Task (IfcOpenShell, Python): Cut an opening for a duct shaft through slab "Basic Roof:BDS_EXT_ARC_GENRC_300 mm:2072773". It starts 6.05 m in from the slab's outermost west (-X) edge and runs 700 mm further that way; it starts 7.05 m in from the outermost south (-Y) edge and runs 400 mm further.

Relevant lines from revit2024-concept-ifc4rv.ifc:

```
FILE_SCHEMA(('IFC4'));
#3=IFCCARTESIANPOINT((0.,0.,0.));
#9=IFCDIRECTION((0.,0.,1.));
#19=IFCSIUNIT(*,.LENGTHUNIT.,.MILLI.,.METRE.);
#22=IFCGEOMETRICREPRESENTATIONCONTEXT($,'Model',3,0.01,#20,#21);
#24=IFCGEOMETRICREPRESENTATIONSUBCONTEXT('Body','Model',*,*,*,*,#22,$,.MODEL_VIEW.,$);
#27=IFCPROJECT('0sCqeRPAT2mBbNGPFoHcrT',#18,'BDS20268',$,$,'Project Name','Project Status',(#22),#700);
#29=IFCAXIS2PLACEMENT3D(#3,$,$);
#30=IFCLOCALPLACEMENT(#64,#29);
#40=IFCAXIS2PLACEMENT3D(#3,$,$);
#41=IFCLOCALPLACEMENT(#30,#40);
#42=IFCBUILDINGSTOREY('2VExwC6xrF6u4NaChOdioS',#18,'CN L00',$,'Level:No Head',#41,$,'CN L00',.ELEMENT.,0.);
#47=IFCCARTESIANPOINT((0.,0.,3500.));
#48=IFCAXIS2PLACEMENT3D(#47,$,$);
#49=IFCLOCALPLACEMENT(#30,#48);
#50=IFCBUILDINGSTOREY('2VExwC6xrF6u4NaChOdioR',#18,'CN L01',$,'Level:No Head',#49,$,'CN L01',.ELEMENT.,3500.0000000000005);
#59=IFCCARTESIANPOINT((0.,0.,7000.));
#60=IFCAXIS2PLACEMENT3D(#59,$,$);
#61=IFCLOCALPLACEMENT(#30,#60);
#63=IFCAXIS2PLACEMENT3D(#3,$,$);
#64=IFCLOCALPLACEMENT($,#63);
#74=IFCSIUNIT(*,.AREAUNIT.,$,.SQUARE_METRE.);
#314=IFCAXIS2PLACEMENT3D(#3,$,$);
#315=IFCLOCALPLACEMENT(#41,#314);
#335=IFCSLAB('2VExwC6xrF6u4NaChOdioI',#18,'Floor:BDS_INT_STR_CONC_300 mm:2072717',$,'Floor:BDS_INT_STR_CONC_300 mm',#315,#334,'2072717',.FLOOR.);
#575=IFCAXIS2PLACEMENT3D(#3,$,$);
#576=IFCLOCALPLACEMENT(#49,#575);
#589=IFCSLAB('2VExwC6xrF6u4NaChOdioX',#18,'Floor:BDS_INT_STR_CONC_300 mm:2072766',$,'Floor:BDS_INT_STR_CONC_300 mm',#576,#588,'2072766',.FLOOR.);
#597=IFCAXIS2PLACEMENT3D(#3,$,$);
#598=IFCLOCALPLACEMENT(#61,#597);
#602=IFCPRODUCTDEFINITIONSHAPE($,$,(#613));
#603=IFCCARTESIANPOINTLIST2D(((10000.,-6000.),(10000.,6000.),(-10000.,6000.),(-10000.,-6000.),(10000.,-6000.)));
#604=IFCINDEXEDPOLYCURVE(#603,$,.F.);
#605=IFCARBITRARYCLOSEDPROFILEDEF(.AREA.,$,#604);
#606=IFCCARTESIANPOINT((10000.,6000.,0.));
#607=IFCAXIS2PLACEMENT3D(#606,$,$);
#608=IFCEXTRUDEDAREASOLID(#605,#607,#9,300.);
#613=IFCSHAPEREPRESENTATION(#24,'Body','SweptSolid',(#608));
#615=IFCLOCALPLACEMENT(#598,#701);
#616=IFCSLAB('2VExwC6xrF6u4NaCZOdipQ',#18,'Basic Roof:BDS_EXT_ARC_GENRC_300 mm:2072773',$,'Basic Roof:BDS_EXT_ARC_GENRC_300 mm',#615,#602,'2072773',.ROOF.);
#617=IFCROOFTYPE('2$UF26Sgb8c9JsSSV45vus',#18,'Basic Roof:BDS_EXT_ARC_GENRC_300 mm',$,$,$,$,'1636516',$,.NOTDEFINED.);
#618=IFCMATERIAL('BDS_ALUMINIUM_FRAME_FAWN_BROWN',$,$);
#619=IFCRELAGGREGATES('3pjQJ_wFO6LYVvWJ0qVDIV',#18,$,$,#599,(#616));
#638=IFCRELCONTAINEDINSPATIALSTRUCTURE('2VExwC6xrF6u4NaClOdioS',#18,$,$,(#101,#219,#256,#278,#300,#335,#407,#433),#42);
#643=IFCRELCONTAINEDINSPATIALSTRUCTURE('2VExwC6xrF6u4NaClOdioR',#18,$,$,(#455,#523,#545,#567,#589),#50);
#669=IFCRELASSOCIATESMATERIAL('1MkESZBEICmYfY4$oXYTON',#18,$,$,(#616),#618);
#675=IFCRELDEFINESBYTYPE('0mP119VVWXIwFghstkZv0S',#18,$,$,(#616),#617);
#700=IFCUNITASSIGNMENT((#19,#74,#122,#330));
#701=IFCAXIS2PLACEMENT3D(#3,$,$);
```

```python
import numpy as np
import ifcopenshell
import ifcopenshell.api.feature
import ifcopenshell.api.geometry
import ifcopenshell.api.root
import ifcopenshell.geom
import ifcopenshell.util.placement
import ifcopenshell.util.representation
import ifcopenshell.util.shape
import ifcopenshell.util.unit

model = ifcopenshell.open("revit2024-concept-ifc4rv.ifc")
unit_scale = ifcopenshell.util.unit.calculate_unit_scale(model)
settings = ifcopenshell.geom.settings()


def volume(element):
    """Net volume in cubic metres, openings subtracted."""
    shape = ifcopenshell.geom.create_shape(settings, element)
    return ifcopenshell.util.shape.get_volume(shape.geometry)


slab = model.by_guid("2VExwC6xrF6u4NaCZOdipQ")
before = volume(slab)

# Extent in the slab's own axes, in metres. The edges named are its -X and -Y sides.
slab_shape = ifcopenshell.geom.create_shape(settings, slab)
vertices = ifcopenshell.util.shape.get_vertices(slab_shape.geometry)
x_min, y_min, bottom = vertices.min(axis=0)
top = vertices[:, 2].max()

opening = ifcopenshell.api.root.create_entity(model, ifc_class="IfcOpeningElement", name="Duct shaft opening", predefined_type="OPENING")
context = ifcopenshell.util.representation.get_context(model, "Model", "Body", "MODEL_VIEW")
width, depth = 0.7, 0.4
outline = [(0.0, 0.0), (width, 0.0), (width, depth), (0.0, depth), (0.0, 0.0)]
# Overshoot both faces by 50 mm so the cut is clean.
shape = ifcopenshell.api.geometry.add_slab_representation(
    model, context=context, depth=top - bottom + 0.1, polyline=outline
)
ifcopenshell.api.geometry.assign_representation(model, product=opening, representation=shape)

matrix = ifcopenshell.util.placement.get_local_placement(slab.ObjectPlacement)
matrix[:, 3] = matrix @ np.append(np.array([x_min + 6.05, y_min + 7.05, bottom - 0.05]) / unit_scale, 1.0)
ifcopenshell.api.geometry.edit_object_placement(model, product=opening, matrix=matrix, is_si=False)
ifcopenshell.api.feature.add_feature(model, feature=opening, element=slab)

after = volume(slab)

print(f"slab volume {before:.3f} -> {after:.3f} m3")

model.write("revit2024-concept-ifc4rv_rev.ifc")
```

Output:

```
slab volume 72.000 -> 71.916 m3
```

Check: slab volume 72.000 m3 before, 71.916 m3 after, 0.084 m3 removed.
